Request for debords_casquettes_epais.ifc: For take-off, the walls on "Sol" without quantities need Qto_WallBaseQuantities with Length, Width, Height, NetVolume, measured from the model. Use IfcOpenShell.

First a look at what the model holds.

```python
import ifcopenshell
import ifcopenshell.util.element
import ifcopenshell.util.unit

model = ifcopenshell.open("debords_casquettes_epais.ifc")
print(model.schema)
for unit_type in ("LENGTHUNIT", "AREAUNIT", "VOLUMEUNIT"):
    print(unit_type, ifcopenshell.util.unit.calculate_unit_scale(model, unit_type))
storey = next(s for s in model.by_type("IfcBuildingStorey") if s.Name == "Sol")
walls = [e for e in ifcopenshell.util.element.get_decomposition(storey) if e.is_a("IfcWall")]
for e in sorted(walls, key=lambda e: e.id()):
    print(e.id(), e.is_a(), e.Name, list(ifcopenshell.util.element.get_psets(e, qtos_only=True)), sep=" | ")
```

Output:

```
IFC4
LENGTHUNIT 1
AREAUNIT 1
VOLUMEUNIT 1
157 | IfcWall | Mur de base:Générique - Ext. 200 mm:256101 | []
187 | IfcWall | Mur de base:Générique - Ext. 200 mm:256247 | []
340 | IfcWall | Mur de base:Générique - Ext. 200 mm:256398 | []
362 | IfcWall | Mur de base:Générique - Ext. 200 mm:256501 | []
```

```python
import ifcopenshell
import ifcopenshell.api.pset
import ifcopenshell.geom
import ifcopenshell.util.element
import ifcopenshell.util.shape
import ifcopenshell.util.unit

model = ifcopenshell.open("debords_casquettes_epais.ifc")
unit_scale = ifcopenshell.util.unit.calculate_unit_scale(model)
volume_scale = ifcopenshell.util.unit.calculate_unit_scale(model, "VOLUMEUNIT")
settings = ifcopenshell.geom.settings()

storey = next(s for s in model.by_type("IfcBuildingStorey") if s.Name == "Sol")
walls = [e for e in ifcopenshell.util.element.get_decomposition(storey) if e.is_a("IfcWall")]

for e in sorted(walls, key=lambda e: e.id()):
    if ifcopenshell.util.element.get_psets(e, qtos_only=True, should_inherit=False):
        continue
    # Geometry comes back in metres, in the element's own axes.
    shape = ifcopenshell.geom.create_shape(settings, e)
    values = {
        "Length": ifcopenshell.util.shape.get_x(shape.geometry) / unit_scale,
        "Width": ifcopenshell.util.shape.get_y(shape.geometry) / unit_scale,
        "Height": ifcopenshell.util.shape.get_z(shape.geometry) / unit_scale,
        "NetVolume": ifcopenshell.util.shape.get_volume(shape.geometry) / volume_scale,
    }
    qto = ifcopenshell.api.pset.add_qto(model, product=e, name="Qto_WallBaseQuantities")
    ifcopenshell.api.pset.edit_qto(model, qto=qto, properties=values)
    print(e.id(), {k: round(v, 3) for k, v in values.items()})

model.write("debords_casquettes_epais_updated.ifc")
```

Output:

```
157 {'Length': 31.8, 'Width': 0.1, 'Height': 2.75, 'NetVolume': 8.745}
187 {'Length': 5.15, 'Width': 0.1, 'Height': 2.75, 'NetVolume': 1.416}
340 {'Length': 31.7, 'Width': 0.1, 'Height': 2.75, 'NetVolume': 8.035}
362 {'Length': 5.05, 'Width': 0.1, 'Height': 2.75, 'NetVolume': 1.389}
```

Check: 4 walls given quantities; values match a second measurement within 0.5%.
